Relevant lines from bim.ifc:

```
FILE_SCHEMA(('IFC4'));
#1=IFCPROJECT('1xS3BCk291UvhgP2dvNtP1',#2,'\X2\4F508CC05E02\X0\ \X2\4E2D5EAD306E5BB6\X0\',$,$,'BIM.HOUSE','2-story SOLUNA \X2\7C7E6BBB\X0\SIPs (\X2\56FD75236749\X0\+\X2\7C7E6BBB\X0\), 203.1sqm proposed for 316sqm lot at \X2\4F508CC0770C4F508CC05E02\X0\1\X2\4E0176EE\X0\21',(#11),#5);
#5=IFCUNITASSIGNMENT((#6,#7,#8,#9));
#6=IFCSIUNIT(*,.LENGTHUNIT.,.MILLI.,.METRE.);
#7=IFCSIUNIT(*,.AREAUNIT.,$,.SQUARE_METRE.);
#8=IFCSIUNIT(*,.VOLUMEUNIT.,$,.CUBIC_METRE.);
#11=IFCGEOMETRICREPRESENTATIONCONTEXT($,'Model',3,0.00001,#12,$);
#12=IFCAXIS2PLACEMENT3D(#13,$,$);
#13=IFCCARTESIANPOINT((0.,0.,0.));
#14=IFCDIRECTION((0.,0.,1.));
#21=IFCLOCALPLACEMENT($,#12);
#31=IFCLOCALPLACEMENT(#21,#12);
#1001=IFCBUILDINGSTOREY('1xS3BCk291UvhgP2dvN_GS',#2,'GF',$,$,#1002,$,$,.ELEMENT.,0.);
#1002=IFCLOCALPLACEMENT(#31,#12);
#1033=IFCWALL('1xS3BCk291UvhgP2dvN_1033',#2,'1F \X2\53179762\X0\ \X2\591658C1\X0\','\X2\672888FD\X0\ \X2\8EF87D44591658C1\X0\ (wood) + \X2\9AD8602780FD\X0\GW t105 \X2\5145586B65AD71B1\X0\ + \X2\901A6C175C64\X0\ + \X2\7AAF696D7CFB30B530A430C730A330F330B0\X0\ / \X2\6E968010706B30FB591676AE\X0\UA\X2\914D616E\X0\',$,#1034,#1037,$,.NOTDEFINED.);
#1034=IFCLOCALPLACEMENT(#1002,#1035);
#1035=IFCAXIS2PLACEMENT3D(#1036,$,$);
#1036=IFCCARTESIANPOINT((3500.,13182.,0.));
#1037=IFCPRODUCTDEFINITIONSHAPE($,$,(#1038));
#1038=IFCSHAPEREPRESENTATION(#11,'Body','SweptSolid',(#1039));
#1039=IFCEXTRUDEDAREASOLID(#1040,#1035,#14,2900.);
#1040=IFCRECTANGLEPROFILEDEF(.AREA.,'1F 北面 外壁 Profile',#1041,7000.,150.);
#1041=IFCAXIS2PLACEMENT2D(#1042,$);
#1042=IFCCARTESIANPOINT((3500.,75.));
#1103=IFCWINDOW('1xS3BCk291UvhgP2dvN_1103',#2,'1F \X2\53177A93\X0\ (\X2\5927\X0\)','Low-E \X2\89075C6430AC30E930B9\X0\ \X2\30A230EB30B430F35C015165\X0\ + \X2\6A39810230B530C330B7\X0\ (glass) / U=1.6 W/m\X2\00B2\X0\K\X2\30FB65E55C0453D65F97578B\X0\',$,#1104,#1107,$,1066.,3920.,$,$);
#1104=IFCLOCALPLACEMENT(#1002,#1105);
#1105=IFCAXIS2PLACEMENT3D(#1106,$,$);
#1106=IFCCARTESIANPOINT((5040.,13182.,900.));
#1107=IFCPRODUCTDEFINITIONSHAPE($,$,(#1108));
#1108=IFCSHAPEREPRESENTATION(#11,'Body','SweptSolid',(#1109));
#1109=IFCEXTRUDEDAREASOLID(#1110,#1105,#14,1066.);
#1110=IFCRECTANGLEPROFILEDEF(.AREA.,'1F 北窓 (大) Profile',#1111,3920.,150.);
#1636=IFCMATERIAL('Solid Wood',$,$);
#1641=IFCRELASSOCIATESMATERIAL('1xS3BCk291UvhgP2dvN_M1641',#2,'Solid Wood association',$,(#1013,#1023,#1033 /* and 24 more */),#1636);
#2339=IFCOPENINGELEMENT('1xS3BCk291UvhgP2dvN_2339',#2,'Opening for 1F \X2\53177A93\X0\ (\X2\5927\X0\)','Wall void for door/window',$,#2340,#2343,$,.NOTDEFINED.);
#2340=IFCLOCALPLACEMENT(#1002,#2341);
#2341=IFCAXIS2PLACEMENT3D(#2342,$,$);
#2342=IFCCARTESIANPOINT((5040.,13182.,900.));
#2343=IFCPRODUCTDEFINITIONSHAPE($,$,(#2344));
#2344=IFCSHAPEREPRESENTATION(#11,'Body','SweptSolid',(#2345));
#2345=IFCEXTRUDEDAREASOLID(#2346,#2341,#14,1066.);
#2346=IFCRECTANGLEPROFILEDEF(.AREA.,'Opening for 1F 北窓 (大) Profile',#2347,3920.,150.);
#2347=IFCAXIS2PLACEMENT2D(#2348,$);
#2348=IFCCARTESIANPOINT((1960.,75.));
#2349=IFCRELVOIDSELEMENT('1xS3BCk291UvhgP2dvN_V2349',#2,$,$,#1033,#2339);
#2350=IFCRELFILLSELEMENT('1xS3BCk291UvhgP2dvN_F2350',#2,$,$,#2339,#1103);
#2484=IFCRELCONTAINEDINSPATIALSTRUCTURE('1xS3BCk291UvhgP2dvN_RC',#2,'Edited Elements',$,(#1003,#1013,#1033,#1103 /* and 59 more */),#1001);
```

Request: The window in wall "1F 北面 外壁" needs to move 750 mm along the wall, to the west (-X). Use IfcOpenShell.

```python
import ifcopenshell
import ifcopenshell.api.geometry
import ifcopenshell.util.placement
import ifcopenshell.util.unit

model = ifcopenshell.open("bim.ifc")
unit_scale = ifcopenshell.util.unit.calculate_unit_scale(model)

window = model.by_guid("1xS3BCk291UvhgP2dvN_1103")
opening = window.FillsVoids[0].RelatingOpeningElement
wall = opening.VoidsElements[0].RelatingBuildingElement

wall_matrix = ifcopenshell.util.placement.get_local_placement(wall.ObjectPlacement)
shift = wall_matrix[:3, 0] * -0.75 / unit_scale
before = ifcopenshell.util.placement.get_local_placement(window.ObjectPlacement)[:3, 3].copy()

# The window is not placed relative to its opening, so move both.
for product in (opening, window):
    matrix = ifcopenshell.util.placement.get_local_placement(product.ObjectPlacement)
    matrix[:3, 3] += shift
    ifcopenshell.api.geometry.edit_object_placement(model, product=product, matrix=matrix, is_si=False)

after = ifcopenshell.util.placement.get_local_placement(window.ObjectPlacement)[:3, 3]
print("window moved by", (after - before).round(3) + 0.0)

model.write("bim_updated.ifc")
```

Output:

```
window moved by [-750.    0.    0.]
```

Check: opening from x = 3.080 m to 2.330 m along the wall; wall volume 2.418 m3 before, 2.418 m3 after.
